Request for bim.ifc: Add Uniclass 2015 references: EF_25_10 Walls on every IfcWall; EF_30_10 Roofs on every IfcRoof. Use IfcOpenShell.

First a look at what the model holds.

```python
import ifcopenshell

model = ifcopenshell.open("bim.ifc")
print(model.schema)
print("classifications:", [c.Name for c in model.by_type("IfcClassification")])
for ifc_class in ("IfcDoor", "IfcRoof", "IfcStair", "IfcWall", "IfcWindow"):
    print(ifc_class, len(model.by_type(ifc_class)))
```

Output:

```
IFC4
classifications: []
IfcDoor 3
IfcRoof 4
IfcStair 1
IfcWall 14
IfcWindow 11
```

```python
import ifcopenshell
import ifcopenshell.api.classification

model = ifcopenshell.open("bim.ifc")

system = ifcopenshell.api.classification.add_classification(model, classification="Uniclass 2015")

codes = {
    "IfcWall": ("EF_25_10", "Walls"),
    "IfcRoof": ("EF_30_10", "Roofs"),
}
for ifc_class, (code, name) in codes.items():
    products = model.by_type(ifc_class)
    ifcopenshell.api.classification.add_reference(
        model, products=products, classification=system, identification=code, name=name
    )
    print(code, len(products))

model.write("bim_edited.ifc")
```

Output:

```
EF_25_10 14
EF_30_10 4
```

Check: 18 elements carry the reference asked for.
